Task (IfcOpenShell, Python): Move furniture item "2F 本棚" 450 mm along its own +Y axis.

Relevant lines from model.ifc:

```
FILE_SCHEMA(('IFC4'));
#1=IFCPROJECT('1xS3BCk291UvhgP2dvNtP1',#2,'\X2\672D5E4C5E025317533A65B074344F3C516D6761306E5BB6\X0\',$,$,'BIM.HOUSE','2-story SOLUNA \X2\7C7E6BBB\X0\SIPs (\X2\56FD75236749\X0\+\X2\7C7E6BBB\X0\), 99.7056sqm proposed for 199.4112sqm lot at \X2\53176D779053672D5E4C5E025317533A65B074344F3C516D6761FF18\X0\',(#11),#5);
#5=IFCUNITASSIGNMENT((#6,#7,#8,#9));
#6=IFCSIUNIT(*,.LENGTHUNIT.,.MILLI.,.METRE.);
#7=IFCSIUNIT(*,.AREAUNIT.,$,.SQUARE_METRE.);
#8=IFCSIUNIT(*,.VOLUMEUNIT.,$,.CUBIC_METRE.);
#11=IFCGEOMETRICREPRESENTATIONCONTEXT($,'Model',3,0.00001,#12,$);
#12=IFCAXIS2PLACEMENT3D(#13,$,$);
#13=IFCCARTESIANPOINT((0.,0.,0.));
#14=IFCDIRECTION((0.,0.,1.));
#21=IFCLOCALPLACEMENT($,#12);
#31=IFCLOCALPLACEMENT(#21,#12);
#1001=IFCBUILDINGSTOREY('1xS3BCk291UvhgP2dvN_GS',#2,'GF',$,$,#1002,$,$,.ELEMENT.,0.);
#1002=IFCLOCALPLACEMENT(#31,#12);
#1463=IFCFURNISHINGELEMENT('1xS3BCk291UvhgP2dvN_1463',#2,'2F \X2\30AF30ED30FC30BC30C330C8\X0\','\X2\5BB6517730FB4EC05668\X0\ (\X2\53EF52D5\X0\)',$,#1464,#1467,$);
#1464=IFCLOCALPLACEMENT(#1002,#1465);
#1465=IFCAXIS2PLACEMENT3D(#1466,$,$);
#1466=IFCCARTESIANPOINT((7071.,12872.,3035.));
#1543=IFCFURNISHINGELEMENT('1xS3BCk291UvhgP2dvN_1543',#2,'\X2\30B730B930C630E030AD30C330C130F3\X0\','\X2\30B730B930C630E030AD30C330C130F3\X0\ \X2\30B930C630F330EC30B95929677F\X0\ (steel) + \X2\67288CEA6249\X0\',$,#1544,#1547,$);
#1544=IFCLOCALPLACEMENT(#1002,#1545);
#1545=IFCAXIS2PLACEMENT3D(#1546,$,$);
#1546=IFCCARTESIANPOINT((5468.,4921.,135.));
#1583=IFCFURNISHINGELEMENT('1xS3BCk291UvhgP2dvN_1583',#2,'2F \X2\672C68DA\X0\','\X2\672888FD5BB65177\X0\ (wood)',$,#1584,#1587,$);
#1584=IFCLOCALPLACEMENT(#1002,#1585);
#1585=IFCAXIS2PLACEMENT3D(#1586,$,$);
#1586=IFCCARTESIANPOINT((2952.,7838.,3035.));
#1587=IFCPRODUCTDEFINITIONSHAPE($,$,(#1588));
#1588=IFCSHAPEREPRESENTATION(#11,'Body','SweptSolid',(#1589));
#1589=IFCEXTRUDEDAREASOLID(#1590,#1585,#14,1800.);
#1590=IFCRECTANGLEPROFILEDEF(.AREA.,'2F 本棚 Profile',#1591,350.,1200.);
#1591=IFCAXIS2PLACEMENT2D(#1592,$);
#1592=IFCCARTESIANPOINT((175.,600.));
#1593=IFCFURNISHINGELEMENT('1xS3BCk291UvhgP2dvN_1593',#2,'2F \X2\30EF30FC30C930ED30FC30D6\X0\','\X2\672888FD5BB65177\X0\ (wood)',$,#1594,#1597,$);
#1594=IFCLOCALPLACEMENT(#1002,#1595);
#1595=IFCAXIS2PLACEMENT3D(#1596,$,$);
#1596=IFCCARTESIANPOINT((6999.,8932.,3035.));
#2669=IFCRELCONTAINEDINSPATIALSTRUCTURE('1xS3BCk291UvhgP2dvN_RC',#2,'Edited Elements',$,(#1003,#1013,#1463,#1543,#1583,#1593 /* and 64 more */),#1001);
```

```python
import ifcopenshell
import ifcopenshell.api.geometry
import ifcopenshell.util.placement
import ifcopenshell.util.unit

model = ifcopenshell.open("model.ifc")
unit_scale = ifcopenshell.util.unit.calculate_unit_scale(model)

item = model.by_guid("1xS3BCk291UvhgP2dvN_1583")
matrix = ifcopenshell.util.placement.get_local_placement(item.ObjectPlacement)
matrix[:3, 3] += matrix[:3, 1] * 0.45 / unit_scale
ifcopenshell.api.geometry.edit_object_placement(model, product=item, matrix=matrix, is_si=False)

print(ifcopenshell.util.placement.get_local_placement(item.ObjectPlacement).round(3) + 0.0)

model.write("model_edited.ifc")
```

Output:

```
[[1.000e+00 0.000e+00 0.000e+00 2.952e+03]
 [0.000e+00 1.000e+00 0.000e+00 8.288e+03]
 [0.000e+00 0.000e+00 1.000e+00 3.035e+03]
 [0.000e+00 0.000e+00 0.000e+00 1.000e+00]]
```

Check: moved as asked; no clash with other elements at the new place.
